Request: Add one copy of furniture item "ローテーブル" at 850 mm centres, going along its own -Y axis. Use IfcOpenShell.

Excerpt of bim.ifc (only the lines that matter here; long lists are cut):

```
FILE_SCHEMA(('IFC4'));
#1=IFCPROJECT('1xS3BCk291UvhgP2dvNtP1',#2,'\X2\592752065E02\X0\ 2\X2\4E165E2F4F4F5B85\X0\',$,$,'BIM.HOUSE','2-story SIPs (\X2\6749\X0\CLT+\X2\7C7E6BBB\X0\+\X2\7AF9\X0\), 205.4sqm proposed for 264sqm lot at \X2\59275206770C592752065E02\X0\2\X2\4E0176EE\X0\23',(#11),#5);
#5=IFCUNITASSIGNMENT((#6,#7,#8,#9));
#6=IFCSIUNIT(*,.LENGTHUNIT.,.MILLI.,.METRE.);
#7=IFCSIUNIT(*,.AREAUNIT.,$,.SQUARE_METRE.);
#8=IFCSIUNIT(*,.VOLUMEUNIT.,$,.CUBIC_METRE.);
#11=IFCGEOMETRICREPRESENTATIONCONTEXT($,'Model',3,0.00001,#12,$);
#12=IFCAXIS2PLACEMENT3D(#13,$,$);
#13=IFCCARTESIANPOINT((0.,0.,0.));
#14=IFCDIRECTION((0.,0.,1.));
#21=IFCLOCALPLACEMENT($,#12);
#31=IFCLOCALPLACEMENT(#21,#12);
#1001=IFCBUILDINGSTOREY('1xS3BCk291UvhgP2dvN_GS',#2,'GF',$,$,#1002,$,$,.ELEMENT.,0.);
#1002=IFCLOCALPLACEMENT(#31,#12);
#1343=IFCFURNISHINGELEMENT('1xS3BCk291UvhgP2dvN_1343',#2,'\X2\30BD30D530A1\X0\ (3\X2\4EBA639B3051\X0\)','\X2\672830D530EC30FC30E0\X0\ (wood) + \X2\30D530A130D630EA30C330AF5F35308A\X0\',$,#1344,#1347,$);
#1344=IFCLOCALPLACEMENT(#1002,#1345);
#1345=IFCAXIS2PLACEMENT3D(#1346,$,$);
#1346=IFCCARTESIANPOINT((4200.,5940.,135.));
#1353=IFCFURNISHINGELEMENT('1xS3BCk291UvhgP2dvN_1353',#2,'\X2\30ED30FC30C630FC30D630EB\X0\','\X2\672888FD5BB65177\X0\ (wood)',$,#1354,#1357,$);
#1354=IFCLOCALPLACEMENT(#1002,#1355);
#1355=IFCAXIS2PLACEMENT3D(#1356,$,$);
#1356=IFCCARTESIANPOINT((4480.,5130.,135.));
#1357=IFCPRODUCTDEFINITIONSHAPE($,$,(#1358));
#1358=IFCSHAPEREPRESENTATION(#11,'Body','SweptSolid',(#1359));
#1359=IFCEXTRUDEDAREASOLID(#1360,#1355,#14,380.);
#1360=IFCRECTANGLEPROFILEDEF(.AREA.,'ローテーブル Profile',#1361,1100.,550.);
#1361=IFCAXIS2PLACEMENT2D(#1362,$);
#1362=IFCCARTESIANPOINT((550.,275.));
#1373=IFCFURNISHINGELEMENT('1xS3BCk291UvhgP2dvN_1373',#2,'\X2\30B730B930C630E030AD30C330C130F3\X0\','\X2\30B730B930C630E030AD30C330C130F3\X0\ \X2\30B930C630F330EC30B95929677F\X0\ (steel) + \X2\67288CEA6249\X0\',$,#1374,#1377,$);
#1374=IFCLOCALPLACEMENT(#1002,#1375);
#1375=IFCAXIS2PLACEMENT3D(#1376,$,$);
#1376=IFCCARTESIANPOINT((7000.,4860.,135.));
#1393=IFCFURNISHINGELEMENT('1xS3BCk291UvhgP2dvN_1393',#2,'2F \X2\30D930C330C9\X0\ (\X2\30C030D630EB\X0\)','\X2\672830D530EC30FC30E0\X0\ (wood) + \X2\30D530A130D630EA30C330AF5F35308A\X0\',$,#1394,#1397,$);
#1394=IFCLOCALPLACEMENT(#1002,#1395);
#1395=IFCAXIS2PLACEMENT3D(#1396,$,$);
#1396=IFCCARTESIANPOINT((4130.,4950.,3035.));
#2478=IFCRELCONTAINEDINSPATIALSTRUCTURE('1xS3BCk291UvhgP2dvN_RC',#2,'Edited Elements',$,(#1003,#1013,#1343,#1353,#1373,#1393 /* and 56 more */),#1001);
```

```python
import ifcopenshell
import ifcopenshell.api.geometry
import ifcopenshell.api.root
import ifcopenshell.util.element
import ifcopenshell.util.placement
import ifcopenshell.util.unit

model = ifcopenshell.open("bim.ifc")
unit_scale = ifcopenshell.util.unit.calculate_unit_scale(model)


def reuse_history(source, copy):
    """copy_class also copies each property set's owner history, people and application; keep the originals."""
    for rel in copy.IsDefinedBy:
        if rel.is_a("IfcRelDefinesByProperties") and (history := rel.RelatingPropertyDefinition.OwnerHistory):
            rel.RelatingPropertyDefinition.OwnerHistory = source.OwnerHistory
            ifcopenshell.util.element.remove_deep2(model, history)


source = model.by_guid("1xS3BCk291UvhgP2dvN_1353")
base = ifcopenshell.util.placement.get_local_placement(source.ObjectPlacement)
step = -base[:3, 1] * 0.85 / unit_scale

for i in range(1, 2):
    copy = ifcopenshell.api.root.copy_class(model, product=source)
    copy.Representation = ifcopenshell.util.element.copy_deep(
        model, source.Representation, exclude=["IfcGeometricRepresentationContext", "IfcRepresentationMap"]
    )
    reuse_history(source, copy)
    matrix = base.copy()
    matrix[:3, 3] += i * step
    print("added at", matrix[:3, 3].round(3) + 0.0)
    ifcopenshell.api.geometry.edit_object_placement(model, product=copy, matrix=matrix, is_si=False)

model.write("bim_updated.ifc")
```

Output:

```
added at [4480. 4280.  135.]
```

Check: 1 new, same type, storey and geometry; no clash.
